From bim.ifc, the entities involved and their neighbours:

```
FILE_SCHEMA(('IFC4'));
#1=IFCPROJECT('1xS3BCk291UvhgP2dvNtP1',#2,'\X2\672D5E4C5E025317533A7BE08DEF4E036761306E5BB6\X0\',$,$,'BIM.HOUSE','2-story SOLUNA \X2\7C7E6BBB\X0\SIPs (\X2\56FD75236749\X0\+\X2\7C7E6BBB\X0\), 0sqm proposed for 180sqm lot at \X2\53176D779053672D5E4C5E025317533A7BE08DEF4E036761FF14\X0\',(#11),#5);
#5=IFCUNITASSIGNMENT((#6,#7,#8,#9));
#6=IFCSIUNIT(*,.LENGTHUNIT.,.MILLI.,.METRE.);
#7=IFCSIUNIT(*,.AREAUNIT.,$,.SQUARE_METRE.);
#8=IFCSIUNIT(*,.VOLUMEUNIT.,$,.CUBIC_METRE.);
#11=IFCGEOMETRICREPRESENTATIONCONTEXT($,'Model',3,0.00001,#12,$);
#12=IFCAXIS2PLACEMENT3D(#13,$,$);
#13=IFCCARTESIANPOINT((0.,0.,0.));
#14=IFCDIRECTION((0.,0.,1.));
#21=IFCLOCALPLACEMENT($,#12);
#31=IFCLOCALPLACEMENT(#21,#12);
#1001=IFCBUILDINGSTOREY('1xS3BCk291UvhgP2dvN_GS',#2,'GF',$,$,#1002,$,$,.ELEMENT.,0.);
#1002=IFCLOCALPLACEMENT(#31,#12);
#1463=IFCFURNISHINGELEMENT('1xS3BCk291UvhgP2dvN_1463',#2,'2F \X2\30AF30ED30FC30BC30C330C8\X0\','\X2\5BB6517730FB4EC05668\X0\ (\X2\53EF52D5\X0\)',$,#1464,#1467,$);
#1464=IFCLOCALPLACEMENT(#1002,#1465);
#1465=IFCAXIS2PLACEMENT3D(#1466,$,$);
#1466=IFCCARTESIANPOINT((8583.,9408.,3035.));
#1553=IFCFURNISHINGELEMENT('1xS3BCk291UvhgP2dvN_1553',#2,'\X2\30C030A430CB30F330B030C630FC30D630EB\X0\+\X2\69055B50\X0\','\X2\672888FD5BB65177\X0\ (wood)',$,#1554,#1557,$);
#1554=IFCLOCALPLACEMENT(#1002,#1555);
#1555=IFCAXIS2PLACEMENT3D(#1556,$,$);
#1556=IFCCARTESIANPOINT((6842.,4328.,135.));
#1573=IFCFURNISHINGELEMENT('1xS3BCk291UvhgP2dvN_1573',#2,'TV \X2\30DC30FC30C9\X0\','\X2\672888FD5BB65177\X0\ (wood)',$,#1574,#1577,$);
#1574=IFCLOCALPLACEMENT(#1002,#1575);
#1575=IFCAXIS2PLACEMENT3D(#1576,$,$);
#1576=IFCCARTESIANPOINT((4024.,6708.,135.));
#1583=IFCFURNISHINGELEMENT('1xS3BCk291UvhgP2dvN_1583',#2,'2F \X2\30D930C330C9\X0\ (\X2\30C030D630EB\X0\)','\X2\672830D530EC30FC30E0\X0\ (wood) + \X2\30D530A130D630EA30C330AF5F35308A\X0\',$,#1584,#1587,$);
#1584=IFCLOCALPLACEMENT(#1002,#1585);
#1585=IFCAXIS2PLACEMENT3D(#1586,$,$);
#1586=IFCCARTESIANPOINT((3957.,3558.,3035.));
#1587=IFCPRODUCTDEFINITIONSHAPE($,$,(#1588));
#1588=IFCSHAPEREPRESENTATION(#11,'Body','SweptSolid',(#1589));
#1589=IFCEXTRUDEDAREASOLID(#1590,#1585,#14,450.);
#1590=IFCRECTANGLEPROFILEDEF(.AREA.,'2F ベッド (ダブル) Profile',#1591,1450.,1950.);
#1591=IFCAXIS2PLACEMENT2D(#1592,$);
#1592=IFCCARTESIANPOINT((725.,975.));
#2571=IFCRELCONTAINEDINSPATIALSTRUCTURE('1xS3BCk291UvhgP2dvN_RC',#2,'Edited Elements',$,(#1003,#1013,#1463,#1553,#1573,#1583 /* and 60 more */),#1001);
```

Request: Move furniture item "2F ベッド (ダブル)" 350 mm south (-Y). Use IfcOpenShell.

```python
import ifcopenshell
import ifcopenshell.api.geometry
import ifcopenshell.util.placement
import ifcopenshell.util.unit

model = ifcopenshell.open("bim.ifc")
unit_scale = ifcopenshell.util.unit.calculate_unit_scale(model)

item = model.by_guid("1xS3BCk291UvhgP2dvN_1583")
matrix = ifcopenshell.util.placement.get_local_placement(item.ObjectPlacement)
matrix[1, 3] -= 0.35 / unit_scale
ifcopenshell.api.geometry.edit_object_placement(model, product=item, matrix=matrix, is_si=False)

print(ifcopenshell.util.placement.get_local_placement(item.ObjectPlacement).round(3) + 0.0)

model.write("bim_edited.ifc")
```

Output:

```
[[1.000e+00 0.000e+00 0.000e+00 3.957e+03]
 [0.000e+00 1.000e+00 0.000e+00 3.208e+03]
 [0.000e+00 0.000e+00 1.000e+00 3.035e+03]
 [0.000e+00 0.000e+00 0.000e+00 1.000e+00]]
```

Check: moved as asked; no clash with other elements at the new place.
